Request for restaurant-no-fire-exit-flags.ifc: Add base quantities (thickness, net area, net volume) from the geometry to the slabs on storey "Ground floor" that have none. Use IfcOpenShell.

First a look at what the model holds.

```python
import ifcopenshell
import ifcopenshell.util.element
import ifcopenshell.util.unit

model = ifcopenshell.open("restaurant-no-fire-exit-flags.ifc")
print(model.schema)
for unit_type in ("LENGTHUNIT", "AREAUNIT", "VOLUMEUNIT"):
    print(unit_type, ifcopenshell.util.unit.calculate_unit_scale(model, unit_type))
storey = next(s for s in model.by_type("IfcBuildingStorey") if s.Name == "Ground floor")
slabs = [e for e in ifcopenshell.util.element.get_decomposition(storey) if e.is_a("IfcSlab")]
for e in sorted(slabs, key=lambda e: e.id()):
    print(e.id(), e.is_a(), e.Name, list(ifcopenshell.util.element.get_psets(e, qtos_only=True)), sep=" | ")
```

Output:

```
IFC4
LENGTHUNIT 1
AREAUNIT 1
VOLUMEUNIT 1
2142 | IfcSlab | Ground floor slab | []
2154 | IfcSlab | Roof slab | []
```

```python
import ifcopenshell
import ifcopenshell.api.pset
import ifcopenshell.geom
import ifcopenshell.util.element
import ifcopenshell.util.shape
import ifcopenshell.util.unit

model = ifcopenshell.open("restaurant-no-fire-exit-flags.ifc")
unit_scale = ifcopenshell.util.unit.calculate_unit_scale(model)
area_scale = ifcopenshell.util.unit.calculate_unit_scale(model, "AREAUNIT")
volume_scale = ifcopenshell.util.unit.calculate_unit_scale(model, "VOLUMEUNIT")
settings = ifcopenshell.geom.settings()

storey = next(s for s in model.by_type("IfcBuildingStorey") if s.Name == "Ground floor")
slabs = [e for e in ifcopenshell.util.element.get_decomposition(storey) if e.is_a("IfcSlab")]

for e in sorted(slabs, key=lambda e: e.id()):
    if ifcopenshell.util.element.get_psets(e, qtos_only=True, should_inherit=False):
        continue
    # Geometry comes back in metres, in the element's own axes.
    shape = ifcopenshell.geom.create_shape(settings, e)
    values = {
        "Width": ifcopenshell.util.shape.get_z(shape.geometry) / unit_scale,
        "NetArea": ifcopenshell.util.shape.get_footprint_area(shape.geometry) / area_scale,
        "NetVolume": ifcopenshell.util.shape.get_volume(shape.geometry) / volume_scale,
    }
    qto = ifcopenshell.api.pset.add_qto(model, product=e, name="Qto_SlabBaseQuantities")
    ifcopenshell.api.pset.edit_qto(model, qto=qto, properties=values)
    print(e.id(), {k: round(v, 3) for k, v in values.items()})

model.write("restaurant-no-fire-exit-flags_v2.ifc")
```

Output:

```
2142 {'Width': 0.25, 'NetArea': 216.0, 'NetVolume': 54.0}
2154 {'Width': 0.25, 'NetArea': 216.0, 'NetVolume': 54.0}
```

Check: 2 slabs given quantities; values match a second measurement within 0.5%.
